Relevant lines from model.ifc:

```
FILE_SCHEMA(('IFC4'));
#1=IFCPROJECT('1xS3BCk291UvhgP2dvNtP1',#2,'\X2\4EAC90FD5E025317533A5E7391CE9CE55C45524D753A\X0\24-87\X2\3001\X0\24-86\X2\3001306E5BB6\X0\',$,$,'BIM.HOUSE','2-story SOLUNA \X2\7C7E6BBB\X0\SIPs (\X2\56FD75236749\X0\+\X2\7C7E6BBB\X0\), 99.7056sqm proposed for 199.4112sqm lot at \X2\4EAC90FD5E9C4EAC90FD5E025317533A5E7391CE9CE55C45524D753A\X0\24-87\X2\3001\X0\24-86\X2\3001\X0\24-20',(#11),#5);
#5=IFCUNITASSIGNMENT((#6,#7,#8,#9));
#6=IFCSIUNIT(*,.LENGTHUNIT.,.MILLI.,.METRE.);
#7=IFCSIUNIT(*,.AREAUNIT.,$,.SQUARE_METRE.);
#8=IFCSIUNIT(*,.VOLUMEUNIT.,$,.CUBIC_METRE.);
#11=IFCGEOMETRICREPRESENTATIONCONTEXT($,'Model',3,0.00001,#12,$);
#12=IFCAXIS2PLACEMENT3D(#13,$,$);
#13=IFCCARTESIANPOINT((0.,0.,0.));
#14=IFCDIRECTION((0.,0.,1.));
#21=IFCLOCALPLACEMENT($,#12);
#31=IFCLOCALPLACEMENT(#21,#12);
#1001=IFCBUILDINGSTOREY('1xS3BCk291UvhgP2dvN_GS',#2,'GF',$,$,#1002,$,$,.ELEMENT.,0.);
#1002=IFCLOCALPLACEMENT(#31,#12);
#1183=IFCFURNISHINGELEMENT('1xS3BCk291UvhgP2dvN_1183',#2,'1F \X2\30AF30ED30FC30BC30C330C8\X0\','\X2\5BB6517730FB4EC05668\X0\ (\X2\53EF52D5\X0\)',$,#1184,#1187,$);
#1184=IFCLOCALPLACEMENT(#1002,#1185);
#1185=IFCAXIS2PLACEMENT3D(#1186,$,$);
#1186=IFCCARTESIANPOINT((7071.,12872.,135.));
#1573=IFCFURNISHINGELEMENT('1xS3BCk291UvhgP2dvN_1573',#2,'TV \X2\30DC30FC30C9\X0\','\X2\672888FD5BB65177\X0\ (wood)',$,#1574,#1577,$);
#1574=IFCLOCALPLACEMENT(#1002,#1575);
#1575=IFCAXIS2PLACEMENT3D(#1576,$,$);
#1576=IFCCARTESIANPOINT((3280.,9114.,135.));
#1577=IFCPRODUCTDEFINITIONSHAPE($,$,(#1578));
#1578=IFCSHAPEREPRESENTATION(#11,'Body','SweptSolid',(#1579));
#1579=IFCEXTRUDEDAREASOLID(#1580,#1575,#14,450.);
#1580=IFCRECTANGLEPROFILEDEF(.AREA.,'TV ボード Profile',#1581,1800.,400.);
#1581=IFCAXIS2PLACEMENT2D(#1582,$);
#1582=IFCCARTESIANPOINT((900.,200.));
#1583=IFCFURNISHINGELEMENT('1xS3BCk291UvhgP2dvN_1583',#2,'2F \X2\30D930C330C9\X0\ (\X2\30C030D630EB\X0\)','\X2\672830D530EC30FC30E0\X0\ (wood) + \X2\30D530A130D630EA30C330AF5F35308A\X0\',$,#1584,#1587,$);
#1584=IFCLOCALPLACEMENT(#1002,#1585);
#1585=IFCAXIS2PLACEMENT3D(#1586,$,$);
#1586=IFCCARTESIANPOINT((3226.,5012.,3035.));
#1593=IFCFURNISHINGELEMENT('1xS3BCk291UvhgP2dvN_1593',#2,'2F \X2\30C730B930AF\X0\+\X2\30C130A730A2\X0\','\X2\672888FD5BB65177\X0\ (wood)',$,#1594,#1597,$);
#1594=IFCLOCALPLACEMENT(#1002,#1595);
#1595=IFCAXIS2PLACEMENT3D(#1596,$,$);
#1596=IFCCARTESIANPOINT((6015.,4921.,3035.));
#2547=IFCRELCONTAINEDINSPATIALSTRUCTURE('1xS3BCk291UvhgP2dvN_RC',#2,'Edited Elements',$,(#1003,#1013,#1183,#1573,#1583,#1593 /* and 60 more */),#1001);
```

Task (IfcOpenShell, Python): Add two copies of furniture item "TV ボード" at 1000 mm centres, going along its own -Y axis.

```python
import ifcopenshell
import ifcopenshell.api.geometry
import ifcopenshell.api.root
import ifcopenshell.util.element
import ifcopenshell.util.placement
import ifcopenshell.util.unit

model = ifcopenshell.open("model.ifc")
unit_scale = ifcopenshell.util.unit.calculate_unit_scale(model)


def reuse_history(source, copy):
    """copy_class also copies each property set's owner history, people and application; keep the originals."""
    for rel in copy.IsDefinedBy:
        if rel.is_a("IfcRelDefinesByProperties") and (history := rel.RelatingPropertyDefinition.OwnerHistory):
            rel.RelatingPropertyDefinition.OwnerHistory = source.OwnerHistory
            ifcopenshell.util.element.remove_deep2(model, history)


source = model.by_guid("1xS3BCk291UvhgP2dvN_1573")
base = ifcopenshell.util.placement.get_local_placement(source.ObjectPlacement)
step = -base[:3, 1] * 1 / unit_scale

for i in range(1, 3):
    copy = ifcopenshell.api.root.copy_class(model, product=source)
    copy.Representation = ifcopenshell.util.element.copy_deep(
        model, source.Representation, exclude=["IfcGeometricRepresentationContext", "IfcRepresentationMap"]
    )
    reuse_history(source, copy)
    matrix = base.copy()
    matrix[:3, 3] += i * step
    print("added at", matrix[:3, 3].round(3) + 0.0)
    ifcopenshell.api.geometry.edit_object_placement(model, product=copy, matrix=matrix, is_si=False)

model.write("model_rev.ifc")
```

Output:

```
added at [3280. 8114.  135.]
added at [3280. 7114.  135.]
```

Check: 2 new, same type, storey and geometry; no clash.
